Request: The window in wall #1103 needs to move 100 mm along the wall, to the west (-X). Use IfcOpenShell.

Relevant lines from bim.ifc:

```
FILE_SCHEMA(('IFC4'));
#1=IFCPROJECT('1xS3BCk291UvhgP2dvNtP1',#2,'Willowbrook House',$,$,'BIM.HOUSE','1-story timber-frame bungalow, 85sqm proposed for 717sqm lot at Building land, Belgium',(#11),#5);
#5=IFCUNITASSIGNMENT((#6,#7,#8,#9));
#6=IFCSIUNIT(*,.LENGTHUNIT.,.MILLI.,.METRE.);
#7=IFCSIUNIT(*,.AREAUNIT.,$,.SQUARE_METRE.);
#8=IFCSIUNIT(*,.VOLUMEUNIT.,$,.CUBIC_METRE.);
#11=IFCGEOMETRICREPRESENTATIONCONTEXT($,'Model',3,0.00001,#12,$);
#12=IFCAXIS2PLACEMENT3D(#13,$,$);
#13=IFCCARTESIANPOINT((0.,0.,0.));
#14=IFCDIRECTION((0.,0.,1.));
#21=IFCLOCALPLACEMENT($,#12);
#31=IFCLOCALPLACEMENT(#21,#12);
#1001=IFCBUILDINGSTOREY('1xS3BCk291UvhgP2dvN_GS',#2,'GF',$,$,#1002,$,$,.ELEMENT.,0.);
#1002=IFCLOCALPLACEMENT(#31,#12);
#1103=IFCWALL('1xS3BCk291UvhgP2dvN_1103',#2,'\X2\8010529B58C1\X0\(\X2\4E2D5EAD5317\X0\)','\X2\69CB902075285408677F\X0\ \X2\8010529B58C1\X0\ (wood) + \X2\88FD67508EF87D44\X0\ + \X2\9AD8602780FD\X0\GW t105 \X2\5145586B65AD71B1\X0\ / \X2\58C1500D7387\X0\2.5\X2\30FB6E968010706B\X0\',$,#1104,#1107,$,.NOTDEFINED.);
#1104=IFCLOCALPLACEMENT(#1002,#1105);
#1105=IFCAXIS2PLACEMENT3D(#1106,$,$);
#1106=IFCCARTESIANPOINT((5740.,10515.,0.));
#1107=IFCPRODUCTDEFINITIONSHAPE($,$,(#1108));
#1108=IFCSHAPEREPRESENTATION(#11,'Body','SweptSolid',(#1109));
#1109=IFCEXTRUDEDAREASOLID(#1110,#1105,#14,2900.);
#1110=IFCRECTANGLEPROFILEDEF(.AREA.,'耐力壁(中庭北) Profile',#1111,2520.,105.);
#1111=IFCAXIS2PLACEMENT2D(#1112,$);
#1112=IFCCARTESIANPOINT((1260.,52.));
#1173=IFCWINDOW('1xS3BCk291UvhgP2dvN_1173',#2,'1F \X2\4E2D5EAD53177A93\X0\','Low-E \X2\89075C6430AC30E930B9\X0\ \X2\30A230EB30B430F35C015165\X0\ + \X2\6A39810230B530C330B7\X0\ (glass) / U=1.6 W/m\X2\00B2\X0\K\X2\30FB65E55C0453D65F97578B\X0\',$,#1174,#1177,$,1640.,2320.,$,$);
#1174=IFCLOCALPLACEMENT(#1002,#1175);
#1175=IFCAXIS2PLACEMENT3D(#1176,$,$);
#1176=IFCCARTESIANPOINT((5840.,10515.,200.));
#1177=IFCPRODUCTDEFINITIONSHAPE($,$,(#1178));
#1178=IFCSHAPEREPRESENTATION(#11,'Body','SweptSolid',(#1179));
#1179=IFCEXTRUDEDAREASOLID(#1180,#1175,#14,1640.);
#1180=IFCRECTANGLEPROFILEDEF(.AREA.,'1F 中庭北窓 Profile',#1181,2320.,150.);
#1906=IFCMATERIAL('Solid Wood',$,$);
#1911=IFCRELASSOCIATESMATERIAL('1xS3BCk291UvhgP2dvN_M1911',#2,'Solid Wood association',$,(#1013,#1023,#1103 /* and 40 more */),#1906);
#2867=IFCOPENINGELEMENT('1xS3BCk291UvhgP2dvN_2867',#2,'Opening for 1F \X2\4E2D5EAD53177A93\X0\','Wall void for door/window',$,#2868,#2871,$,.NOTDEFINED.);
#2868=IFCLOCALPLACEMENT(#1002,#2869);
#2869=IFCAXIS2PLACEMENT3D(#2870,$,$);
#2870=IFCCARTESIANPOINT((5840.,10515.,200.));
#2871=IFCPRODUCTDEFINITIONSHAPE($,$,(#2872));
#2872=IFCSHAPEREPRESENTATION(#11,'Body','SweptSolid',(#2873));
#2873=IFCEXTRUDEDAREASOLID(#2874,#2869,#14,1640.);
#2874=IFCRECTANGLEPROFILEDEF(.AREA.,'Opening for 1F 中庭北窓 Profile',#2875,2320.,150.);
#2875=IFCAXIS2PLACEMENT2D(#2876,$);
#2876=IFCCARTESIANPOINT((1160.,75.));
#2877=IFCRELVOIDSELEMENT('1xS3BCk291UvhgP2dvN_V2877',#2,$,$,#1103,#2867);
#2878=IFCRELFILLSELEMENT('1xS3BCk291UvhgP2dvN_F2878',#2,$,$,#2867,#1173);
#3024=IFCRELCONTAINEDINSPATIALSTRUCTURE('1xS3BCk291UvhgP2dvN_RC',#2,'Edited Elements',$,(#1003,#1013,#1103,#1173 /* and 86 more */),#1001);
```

```python
import ifcopenshell
import ifcopenshell.api.geometry
import ifcopenshell.util.placement

model = ifcopenshell.open("bim.ifc")

window = model.by_guid("1xS3BCk291UvhgP2dvN_1173")
opening = window.FillsVoids[0].RelatingOpeningElement
wall = opening.VoidsElements[0].RelatingBuildingElement

wall_matrix = ifcopenshell.util.placement.get_local_placement(wall.ObjectPlacement)
shift = wall_matrix[:3, 0] * -100.0
before = ifcopenshell.util.placement.get_local_placement(window.ObjectPlacement)[:3, 3].copy()

# The window is not placed relative to its opening, so move both.
for product in (opening, window):
    matrix = ifcopenshell.util.placement.get_local_placement(product.ObjectPlacement)
    matrix[:3, 3] += shift
    ifcopenshell.api.geometry.edit_object_placement(model, product=product, matrix=matrix, is_si=False)

after = ifcopenshell.util.placement.get_local_placement(window.ObjectPlacement)[:3, 3]
print("window moved by", (after - before).round(3) + 0.0)

model.write("bim-out.ifc")
```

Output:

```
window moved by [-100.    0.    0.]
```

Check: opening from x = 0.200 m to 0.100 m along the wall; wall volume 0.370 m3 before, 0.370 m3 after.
